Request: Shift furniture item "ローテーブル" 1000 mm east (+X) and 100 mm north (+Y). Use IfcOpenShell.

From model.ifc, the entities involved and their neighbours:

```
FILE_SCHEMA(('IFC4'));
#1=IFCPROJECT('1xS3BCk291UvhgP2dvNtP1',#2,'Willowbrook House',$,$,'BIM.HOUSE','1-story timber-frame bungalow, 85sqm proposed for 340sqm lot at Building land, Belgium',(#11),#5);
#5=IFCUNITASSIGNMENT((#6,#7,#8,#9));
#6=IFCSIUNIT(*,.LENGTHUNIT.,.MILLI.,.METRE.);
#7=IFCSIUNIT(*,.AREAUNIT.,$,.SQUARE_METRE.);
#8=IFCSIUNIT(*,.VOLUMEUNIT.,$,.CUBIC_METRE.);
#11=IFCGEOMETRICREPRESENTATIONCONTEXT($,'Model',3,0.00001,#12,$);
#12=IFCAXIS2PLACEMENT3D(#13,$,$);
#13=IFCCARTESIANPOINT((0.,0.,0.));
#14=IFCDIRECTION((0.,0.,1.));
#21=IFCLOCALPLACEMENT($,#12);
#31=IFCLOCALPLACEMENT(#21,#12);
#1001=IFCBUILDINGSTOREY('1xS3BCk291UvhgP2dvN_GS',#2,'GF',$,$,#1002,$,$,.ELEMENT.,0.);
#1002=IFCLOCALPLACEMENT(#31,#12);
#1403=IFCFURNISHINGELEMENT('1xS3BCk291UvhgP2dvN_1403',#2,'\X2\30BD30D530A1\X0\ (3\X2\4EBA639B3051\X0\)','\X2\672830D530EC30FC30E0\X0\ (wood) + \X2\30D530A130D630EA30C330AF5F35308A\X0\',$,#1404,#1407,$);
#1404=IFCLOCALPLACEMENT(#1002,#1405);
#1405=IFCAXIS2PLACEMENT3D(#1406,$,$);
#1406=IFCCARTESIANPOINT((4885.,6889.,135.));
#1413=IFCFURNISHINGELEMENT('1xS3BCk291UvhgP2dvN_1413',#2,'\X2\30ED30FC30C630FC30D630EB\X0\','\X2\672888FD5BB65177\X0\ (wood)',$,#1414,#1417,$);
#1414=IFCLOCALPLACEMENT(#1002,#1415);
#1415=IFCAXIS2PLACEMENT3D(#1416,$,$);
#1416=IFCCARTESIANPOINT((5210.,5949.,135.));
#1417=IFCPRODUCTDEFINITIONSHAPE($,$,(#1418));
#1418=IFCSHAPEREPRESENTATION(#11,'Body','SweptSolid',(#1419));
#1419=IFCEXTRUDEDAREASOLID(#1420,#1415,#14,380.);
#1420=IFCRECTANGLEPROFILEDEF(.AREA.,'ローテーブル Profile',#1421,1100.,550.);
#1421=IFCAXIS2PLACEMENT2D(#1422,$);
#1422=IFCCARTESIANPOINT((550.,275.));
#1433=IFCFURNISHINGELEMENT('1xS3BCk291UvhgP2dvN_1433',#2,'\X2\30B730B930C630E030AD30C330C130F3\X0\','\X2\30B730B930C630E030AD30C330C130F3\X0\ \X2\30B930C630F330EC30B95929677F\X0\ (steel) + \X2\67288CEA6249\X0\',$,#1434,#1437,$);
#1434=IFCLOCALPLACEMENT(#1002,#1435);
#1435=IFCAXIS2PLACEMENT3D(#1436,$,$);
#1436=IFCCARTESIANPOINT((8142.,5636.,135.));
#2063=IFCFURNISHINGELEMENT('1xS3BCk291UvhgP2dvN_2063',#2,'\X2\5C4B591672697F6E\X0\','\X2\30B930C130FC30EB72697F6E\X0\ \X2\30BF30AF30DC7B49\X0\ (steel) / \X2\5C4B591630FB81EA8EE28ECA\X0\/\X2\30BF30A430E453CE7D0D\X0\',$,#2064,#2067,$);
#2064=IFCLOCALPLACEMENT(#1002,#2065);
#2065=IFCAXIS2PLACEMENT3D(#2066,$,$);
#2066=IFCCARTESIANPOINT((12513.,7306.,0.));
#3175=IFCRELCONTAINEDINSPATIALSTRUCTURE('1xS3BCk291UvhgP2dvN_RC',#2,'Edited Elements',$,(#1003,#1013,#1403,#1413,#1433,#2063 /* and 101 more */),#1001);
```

```python
import ifcopenshell
import ifcopenshell.api.geometry
import ifcopenshell.util.placement
import ifcopenshell.util.unit

model = ifcopenshell.open("model.ifc")
unit_scale = ifcopenshell.util.unit.calculate_unit_scale(model)

item = model.by_id(1413)
matrix = ifcopenshell.util.placement.get_local_placement(item.ObjectPlacement)
matrix[0, 3] += 1 / unit_scale
matrix[1, 3] += 0.1 / unit_scale
ifcopenshell.api.geometry.edit_object_placement(model, product=item, matrix=matrix, is_si=False)

print(ifcopenshell.util.placement.get_local_placement(item.ObjectPlacement).round(3) + 0.0)

model.write("model-out.ifc")
```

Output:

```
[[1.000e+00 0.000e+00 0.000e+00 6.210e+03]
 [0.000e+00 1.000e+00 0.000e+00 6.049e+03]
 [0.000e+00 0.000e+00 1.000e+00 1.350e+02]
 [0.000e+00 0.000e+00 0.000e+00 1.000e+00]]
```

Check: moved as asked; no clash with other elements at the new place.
